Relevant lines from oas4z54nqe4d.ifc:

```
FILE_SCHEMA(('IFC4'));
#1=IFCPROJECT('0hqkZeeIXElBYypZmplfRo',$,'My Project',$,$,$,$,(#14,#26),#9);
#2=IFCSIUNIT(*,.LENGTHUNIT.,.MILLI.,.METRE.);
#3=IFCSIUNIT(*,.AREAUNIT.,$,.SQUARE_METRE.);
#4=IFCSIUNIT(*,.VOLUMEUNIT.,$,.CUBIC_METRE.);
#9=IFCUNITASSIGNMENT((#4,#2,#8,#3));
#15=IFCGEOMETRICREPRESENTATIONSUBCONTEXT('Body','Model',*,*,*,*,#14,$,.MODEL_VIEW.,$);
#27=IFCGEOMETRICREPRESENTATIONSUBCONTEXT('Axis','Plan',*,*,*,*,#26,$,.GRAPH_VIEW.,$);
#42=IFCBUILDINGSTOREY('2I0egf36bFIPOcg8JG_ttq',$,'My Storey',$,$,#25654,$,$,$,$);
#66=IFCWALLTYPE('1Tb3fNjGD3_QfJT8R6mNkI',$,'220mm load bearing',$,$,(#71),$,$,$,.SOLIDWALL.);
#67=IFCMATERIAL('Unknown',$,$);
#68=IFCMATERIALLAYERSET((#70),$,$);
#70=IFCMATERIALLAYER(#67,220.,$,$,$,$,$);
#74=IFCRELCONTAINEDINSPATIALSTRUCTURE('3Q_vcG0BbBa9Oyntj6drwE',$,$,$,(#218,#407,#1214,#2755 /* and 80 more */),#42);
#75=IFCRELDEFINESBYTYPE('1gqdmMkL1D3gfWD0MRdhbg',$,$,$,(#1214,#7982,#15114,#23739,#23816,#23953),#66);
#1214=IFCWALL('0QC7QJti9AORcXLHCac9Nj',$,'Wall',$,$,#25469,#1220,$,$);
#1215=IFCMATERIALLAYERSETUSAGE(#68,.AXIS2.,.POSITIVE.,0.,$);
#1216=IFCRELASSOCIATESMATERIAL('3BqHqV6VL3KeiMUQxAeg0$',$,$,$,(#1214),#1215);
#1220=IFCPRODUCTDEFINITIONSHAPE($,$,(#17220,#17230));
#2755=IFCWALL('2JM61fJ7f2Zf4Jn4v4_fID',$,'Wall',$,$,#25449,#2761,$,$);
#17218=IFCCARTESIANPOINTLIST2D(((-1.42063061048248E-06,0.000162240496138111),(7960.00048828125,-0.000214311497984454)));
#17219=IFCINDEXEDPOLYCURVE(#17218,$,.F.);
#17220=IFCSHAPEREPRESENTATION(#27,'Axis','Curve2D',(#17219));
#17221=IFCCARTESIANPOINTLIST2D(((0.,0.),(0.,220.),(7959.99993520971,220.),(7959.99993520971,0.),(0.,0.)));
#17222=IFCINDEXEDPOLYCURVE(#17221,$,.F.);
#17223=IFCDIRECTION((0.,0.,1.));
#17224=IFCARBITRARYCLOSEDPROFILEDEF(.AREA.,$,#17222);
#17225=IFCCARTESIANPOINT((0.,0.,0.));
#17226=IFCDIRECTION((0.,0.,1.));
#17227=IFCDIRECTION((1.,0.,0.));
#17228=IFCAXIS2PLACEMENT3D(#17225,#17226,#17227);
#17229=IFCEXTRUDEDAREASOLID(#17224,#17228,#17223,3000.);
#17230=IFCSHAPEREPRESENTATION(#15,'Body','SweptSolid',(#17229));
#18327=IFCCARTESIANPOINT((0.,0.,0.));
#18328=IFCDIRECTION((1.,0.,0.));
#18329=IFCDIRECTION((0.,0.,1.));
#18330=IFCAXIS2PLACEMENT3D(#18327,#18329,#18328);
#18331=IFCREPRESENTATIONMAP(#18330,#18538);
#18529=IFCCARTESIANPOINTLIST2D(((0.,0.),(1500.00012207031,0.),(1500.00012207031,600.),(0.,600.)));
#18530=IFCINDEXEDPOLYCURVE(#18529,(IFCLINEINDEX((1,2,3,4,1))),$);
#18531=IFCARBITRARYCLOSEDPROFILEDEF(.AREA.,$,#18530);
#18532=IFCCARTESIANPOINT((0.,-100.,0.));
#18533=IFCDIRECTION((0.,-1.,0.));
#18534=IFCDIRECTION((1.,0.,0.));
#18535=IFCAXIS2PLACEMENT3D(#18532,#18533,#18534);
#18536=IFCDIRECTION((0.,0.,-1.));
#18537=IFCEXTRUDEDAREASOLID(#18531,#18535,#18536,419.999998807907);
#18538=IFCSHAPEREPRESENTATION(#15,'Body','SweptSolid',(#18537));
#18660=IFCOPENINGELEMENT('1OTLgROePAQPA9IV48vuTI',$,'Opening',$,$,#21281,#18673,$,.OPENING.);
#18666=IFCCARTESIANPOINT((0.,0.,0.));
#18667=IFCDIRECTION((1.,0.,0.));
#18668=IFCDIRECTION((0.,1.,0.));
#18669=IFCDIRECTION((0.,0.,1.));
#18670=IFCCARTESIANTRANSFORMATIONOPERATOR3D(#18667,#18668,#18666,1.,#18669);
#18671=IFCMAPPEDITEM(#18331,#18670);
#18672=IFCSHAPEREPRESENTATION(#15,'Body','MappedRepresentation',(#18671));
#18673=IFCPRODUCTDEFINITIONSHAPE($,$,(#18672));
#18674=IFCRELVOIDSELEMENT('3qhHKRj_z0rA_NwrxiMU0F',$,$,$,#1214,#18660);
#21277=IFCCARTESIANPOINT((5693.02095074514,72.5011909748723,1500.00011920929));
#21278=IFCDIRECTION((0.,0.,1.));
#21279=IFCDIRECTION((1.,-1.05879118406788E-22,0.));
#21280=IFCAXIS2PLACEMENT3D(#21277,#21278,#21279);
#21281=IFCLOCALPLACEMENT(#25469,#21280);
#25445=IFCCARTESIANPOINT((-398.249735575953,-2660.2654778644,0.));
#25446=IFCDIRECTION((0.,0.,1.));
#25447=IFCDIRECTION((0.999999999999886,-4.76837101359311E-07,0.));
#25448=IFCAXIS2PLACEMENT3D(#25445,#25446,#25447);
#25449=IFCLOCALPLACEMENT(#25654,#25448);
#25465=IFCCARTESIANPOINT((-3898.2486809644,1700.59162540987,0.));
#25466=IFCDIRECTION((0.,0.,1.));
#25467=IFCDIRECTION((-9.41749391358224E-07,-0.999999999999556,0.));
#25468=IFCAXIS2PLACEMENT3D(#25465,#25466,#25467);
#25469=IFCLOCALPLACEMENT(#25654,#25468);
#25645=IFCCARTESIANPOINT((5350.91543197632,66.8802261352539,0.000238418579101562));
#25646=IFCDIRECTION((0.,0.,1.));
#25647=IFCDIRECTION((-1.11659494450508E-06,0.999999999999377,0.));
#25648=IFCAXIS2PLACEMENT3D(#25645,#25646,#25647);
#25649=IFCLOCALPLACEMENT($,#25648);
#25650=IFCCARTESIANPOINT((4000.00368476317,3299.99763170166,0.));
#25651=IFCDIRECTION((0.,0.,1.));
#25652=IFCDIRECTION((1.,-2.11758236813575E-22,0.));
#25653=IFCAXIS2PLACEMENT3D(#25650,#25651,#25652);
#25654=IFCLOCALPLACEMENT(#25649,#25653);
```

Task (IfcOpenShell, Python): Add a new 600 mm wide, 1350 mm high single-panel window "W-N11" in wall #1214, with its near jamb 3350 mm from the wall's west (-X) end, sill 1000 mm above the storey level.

```python
import numpy as np
import ifcopenshell
import ifcopenshell.api.feature
import ifcopenshell.api.geometry
import ifcopenshell.api.root
import ifcopenshell.api.spatial
import ifcopenshell.geom
import ifcopenshell.util.element
import ifcopenshell.util.placement
import ifcopenshell.util.representation
import ifcopenshell.util.shape
import ifcopenshell.util.unit

model = ifcopenshell.open("oas4z54nqe4d.ifc")
unit_scale = ifcopenshell.util.unit.calculate_unit_scale(model)
settings = ifcopenshell.geom.settings()


def volume(element):
    """Net volume in cubic metres, openings subtracted."""
    shape = ifcopenshell.geom.create_shape(settings, element)
    return ifcopenshell.util.shape.get_volume(shape.geometry)


wall = model.by_guid("0QC7QJti9AORcXLHCac9Nj")
storey = ifcopenshell.util.element.get_container(wall, ifc_class="IfcBuildingStorey")
context = ifcopenshell.util.representation.get_context(model, "Model", "Body", "MODEL_VIEW")
before = volume(wall)

width, height, from_end, sill = 0.6, 1.35, 3.35, 1  # metres

# The wall runs along its own X axis, and the end named is its -X end.
wall_shape = ifcopenshell.geom.create_shape(settings, wall)
x, y, z = ifcopenshell.util.shape.get_vertices(wall_shape.geometry).T
start = x.min() + from_end
face, thickness = float(y.min()), float(y.max() - y.min())
wall_matrix = ifcopenshell.util.placement.get_local_placement(wall.ObjectPlacement)
level = ifcopenshell.util.placement.get_local_placement(storey.ObjectPlacement)[2, 3]


def in_wall(x, y):
    """Placement at x, y metres in the wall's axes, at sill height."""
    matrix = wall_matrix.copy()
    matrix[:, 3] = wall_matrix @ np.array([x / unit_scale, y / unit_scale, 0.0, 1.0])
    matrix[2, 3] = level + sill / unit_scale
    return matrix


# Opening: a box that overshoots both wall faces by 50 mm.
opening = ifcopenshell.api.root.create_entity(model, ifc_class="IfcOpeningElement", predefined_type="OPENING")
box = ifcopenshell.api.geometry.add_wall_representation(
    model, context=context, length=width, height=height, thickness=thickness + 0.1
)
ifcopenshell.api.geometry.assign_representation(model, product=opening, representation=box)
ifcopenshell.api.geometry.edit_object_placement(model, product=opening, matrix=in_wall(start, face - 0.05), is_si=False)
ifcopenshell.api.feature.add_feature(model, feature=opening, element=wall)

window = ifcopenshell.api.root.create_entity(model, ifc_class="IfcWindow", name="W-N11", predefined_type="WINDOW")
window.OverallWidth, window.OverallHeight = width / unit_scale, height / unit_scale
window.PartitioningType = "SINGLE_PANEL"
body = ifcopenshell.api.geometry.add_window_representation(
    model,
    context=context,
    overall_width=window.OverallWidth,
    overall_height=window.OverallHeight,
    partition_type="SINGLE_PANEL",
)
ifcopenshell.api.geometry.assign_representation(model, product=window, representation=body)
ifcopenshell.api.spatial.assign_container(model, products=[window], relating_structure=storey)
ifcopenshell.api.feature.add_filling(model, opening=opening, element=window)

# Centre the window in the wall's thickness.
ifcopenshell.api.geometry.edit_object_placement(model, product=window, matrix=in_wall(start, face), is_si=False)
window_shape = ifcopenshell.geom.create_shape(settings, window)
depth = ifcopenshell.util.shape.get_vertices(window_shape.geometry)[:, 1]
offset = face + thickness / 2 - (depth.min() + depth.max()) / 2
ifcopenshell.api.geometry.edit_object_placement(model, product=window, matrix=in_wall(start, offset), is_si=False)

after = volume(wall)

print(f"wall volume {before:.3f} -> {after:.3f} m3")

model.write("oas4z54nqe4d_v2.ifc")
```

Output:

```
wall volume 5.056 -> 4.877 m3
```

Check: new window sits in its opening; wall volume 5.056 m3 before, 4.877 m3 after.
